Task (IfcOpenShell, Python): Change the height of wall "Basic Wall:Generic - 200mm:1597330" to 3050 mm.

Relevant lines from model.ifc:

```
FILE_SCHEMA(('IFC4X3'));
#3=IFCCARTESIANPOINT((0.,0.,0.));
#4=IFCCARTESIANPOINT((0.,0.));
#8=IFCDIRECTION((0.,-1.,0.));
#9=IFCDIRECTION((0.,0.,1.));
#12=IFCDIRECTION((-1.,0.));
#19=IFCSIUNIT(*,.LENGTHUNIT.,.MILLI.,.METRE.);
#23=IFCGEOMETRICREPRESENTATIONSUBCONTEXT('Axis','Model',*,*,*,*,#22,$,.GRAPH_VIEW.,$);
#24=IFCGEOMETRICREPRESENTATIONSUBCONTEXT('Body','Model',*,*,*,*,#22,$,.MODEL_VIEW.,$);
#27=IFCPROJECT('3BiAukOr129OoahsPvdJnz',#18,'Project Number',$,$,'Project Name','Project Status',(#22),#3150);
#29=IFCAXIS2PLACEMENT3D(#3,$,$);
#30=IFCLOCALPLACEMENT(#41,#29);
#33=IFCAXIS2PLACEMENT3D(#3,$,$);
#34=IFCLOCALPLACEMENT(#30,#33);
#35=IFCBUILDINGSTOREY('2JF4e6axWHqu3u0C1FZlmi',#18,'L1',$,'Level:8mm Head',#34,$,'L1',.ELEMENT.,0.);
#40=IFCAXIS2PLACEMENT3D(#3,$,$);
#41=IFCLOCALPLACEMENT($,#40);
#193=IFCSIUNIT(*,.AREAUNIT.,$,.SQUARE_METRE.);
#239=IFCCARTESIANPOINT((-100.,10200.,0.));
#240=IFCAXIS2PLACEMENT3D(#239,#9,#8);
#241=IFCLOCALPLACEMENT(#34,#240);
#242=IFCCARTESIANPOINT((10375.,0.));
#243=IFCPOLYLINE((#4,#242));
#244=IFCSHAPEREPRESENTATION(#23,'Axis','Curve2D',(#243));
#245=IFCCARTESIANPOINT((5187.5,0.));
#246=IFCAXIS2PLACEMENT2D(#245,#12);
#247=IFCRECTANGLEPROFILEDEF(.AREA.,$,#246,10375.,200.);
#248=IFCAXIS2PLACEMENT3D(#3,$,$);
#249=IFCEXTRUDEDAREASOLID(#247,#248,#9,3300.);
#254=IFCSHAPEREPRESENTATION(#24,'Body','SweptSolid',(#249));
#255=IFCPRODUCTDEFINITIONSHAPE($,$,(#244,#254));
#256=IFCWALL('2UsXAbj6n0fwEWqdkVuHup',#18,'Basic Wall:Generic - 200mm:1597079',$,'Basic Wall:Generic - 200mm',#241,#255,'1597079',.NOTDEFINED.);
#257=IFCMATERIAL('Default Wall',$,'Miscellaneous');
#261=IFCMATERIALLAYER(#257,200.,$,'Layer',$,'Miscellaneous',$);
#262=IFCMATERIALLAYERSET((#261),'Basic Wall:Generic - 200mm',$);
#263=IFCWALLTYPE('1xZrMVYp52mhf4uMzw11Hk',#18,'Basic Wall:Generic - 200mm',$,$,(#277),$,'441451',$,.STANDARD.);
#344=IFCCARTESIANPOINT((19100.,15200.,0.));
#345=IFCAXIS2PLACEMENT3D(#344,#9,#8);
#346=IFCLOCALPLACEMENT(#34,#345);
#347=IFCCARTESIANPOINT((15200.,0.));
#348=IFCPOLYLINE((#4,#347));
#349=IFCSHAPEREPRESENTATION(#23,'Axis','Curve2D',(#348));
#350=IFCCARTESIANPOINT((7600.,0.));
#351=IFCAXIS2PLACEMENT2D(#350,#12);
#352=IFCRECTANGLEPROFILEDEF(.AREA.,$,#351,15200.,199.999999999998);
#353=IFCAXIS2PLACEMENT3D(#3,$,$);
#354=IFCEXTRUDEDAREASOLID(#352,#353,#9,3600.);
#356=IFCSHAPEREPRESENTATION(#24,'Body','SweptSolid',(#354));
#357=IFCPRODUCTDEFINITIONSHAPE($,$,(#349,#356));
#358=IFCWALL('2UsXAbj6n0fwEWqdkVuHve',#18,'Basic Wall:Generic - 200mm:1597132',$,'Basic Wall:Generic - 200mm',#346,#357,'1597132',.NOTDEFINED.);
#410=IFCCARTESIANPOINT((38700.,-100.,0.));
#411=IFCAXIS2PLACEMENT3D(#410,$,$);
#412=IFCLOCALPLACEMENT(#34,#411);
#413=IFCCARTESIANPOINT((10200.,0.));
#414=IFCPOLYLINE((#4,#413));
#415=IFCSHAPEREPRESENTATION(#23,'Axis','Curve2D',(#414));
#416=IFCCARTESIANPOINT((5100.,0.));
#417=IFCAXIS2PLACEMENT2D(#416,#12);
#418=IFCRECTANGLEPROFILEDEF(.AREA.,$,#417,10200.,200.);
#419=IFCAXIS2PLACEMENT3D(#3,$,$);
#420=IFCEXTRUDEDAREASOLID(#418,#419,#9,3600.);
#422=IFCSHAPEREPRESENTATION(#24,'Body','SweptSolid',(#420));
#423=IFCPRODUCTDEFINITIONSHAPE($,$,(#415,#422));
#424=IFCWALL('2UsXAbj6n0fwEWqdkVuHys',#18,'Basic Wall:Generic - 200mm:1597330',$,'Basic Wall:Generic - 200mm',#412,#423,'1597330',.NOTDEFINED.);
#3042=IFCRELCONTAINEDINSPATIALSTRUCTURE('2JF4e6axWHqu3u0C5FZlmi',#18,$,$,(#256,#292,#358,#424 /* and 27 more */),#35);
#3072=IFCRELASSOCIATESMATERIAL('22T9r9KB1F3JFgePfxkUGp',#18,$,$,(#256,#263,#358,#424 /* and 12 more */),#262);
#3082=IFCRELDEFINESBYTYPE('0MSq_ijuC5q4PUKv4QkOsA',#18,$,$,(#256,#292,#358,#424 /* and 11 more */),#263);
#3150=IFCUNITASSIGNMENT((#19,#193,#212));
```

```python
import ifcopenshell
import ifcopenshell.geom
import ifcopenshell.util.representation
import ifcopenshell.util.shape
import ifcopenshell.util.unit

model = ifcopenshell.open("model.ifc")
unit_scale = ifcopenshell.util.unit.calculate_unit_scale(model)
settings = ifcopenshell.geom.settings()


def volume(element):
    """Net volume in cubic metres, openings subtracted."""
    shape = ifcopenshell.geom.create_shape(settings, element)
    return ifcopenshell.util.shape.get_volume(shape.geometry)


wall = model.by_guid("2UsXAbj6n0fwEWqdkVuHys")
before = volume(wall)

body = ifcopenshell.util.representation.get_representation(wall, "Model", "Body")
solid = body.Items[0]
old_height = solid.Depth
solid.Depth = 3.05 / unit_scale
after = volume(wall)

print(f"height {old_height:g} -> {solid.Depth:g}, volume {before:.3f} -> {after:.3f} m3")

model.write("model-out.ifc")
```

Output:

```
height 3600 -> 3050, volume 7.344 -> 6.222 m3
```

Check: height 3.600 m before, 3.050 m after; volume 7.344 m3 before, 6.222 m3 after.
